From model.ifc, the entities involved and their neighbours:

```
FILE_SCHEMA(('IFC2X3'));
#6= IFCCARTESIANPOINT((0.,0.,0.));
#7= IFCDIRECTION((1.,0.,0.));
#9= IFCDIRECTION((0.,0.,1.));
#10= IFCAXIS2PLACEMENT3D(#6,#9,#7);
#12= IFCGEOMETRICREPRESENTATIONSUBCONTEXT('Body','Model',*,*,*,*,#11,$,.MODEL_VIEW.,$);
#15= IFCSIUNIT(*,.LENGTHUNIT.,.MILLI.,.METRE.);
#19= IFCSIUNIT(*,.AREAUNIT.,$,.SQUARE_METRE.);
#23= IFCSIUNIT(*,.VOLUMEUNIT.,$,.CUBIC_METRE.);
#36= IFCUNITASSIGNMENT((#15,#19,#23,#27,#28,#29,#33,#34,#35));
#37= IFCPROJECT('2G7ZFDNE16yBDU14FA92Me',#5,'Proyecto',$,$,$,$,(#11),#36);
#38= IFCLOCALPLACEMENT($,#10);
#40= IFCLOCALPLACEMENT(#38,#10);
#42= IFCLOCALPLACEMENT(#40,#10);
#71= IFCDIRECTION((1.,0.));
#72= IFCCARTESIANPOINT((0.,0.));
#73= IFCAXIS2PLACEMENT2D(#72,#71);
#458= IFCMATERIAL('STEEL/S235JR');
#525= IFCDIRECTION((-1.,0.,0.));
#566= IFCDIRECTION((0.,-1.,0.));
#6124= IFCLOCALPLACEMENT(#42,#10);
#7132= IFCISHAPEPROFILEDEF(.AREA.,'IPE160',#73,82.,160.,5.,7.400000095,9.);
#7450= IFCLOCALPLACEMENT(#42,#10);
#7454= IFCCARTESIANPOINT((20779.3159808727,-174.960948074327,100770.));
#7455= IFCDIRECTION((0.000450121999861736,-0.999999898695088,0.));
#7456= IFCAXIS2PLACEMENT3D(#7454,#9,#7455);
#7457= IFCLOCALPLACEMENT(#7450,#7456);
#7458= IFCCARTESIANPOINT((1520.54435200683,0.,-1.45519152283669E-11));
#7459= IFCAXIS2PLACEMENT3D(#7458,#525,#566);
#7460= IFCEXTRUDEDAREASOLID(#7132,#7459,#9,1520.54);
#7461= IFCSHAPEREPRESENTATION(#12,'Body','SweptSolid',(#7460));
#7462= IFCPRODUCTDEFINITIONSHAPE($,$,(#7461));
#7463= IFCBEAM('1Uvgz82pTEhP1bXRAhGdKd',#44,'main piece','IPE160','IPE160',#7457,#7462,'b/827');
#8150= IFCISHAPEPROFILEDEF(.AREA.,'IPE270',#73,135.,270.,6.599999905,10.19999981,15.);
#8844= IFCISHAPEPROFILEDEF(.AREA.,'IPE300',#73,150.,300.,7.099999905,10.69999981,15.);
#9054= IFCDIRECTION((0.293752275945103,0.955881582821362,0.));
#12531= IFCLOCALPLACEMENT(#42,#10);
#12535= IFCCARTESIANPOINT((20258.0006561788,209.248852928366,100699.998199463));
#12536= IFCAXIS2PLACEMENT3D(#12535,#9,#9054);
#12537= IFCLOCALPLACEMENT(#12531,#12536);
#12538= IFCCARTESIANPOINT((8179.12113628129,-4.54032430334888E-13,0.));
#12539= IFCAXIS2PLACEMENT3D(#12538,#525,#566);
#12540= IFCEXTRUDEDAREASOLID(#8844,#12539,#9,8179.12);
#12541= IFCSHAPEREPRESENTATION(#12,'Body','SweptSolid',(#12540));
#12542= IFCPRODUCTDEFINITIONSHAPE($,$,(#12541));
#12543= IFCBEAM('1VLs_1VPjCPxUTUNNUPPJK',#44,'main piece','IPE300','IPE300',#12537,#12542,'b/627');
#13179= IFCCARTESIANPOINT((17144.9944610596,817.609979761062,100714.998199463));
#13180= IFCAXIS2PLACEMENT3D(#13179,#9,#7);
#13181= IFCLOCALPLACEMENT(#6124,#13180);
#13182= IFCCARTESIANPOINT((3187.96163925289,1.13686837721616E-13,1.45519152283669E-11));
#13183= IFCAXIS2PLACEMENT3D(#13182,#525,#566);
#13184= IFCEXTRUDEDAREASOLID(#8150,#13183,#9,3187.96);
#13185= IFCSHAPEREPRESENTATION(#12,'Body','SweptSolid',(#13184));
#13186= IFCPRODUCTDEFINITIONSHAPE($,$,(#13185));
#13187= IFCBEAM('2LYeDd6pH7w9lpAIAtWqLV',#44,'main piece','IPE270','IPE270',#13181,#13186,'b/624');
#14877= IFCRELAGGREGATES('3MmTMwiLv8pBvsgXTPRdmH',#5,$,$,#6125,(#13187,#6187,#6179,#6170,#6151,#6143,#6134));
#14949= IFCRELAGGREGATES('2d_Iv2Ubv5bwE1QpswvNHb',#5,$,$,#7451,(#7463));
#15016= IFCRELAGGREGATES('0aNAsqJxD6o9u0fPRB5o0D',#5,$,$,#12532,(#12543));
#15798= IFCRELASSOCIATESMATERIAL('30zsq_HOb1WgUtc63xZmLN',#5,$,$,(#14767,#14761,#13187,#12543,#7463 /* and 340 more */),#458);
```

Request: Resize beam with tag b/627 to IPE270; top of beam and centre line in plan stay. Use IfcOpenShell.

```python
import ifcopenshell
import ifcopenshell.util.element
import ifcopenshell.util.representation

model = ifcopenshell.open("model.ifc")

member = model.by_id(12543)
source = next(p for p in model.by_type("IfcIShapeProfileDef") if p.ProfileName == "IPE270")

body = ifcopenshell.util.representation.get_representation(member, "Model", "Body")
solid = body.Items[0]
old_profile = solid.SweptArea

# Copy the section's sizes but keep this member's own profile position.
profile = ifcopenshell.util.element.copy(model, source)
# Profiles are centred, so shift by half the change in depth to hold the top.
shift = (old_profile.OverallDepth - profile.OverallDepth) / 2
x, y = old_profile.Position.Location.Coordinates
up = (0.0, 1.0)  # upwards, in the solid's own plane
location = model.createIfcCartesianPoint((x + up[0] * shift, y + up[1] * shift))
profile.Position = model.createIfcAxis2Placement2D(location, old_profile.Position.RefDirection)
solid.SweptArea = profile
if not model.get_total_inverses(old_profile):
    ifcopenshell.util.element.remove_deep2(model, old_profile)
member.Description = member.Description.replace("IPE300", "IPE270")
member.ObjectType = member.ObjectType.replace("IPE300", "IPE270")

print(solid.SweptArea)

model.write("model_edited.ifc")
```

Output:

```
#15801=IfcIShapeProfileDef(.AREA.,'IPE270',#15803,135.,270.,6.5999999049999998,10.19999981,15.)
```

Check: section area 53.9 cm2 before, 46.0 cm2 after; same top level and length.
